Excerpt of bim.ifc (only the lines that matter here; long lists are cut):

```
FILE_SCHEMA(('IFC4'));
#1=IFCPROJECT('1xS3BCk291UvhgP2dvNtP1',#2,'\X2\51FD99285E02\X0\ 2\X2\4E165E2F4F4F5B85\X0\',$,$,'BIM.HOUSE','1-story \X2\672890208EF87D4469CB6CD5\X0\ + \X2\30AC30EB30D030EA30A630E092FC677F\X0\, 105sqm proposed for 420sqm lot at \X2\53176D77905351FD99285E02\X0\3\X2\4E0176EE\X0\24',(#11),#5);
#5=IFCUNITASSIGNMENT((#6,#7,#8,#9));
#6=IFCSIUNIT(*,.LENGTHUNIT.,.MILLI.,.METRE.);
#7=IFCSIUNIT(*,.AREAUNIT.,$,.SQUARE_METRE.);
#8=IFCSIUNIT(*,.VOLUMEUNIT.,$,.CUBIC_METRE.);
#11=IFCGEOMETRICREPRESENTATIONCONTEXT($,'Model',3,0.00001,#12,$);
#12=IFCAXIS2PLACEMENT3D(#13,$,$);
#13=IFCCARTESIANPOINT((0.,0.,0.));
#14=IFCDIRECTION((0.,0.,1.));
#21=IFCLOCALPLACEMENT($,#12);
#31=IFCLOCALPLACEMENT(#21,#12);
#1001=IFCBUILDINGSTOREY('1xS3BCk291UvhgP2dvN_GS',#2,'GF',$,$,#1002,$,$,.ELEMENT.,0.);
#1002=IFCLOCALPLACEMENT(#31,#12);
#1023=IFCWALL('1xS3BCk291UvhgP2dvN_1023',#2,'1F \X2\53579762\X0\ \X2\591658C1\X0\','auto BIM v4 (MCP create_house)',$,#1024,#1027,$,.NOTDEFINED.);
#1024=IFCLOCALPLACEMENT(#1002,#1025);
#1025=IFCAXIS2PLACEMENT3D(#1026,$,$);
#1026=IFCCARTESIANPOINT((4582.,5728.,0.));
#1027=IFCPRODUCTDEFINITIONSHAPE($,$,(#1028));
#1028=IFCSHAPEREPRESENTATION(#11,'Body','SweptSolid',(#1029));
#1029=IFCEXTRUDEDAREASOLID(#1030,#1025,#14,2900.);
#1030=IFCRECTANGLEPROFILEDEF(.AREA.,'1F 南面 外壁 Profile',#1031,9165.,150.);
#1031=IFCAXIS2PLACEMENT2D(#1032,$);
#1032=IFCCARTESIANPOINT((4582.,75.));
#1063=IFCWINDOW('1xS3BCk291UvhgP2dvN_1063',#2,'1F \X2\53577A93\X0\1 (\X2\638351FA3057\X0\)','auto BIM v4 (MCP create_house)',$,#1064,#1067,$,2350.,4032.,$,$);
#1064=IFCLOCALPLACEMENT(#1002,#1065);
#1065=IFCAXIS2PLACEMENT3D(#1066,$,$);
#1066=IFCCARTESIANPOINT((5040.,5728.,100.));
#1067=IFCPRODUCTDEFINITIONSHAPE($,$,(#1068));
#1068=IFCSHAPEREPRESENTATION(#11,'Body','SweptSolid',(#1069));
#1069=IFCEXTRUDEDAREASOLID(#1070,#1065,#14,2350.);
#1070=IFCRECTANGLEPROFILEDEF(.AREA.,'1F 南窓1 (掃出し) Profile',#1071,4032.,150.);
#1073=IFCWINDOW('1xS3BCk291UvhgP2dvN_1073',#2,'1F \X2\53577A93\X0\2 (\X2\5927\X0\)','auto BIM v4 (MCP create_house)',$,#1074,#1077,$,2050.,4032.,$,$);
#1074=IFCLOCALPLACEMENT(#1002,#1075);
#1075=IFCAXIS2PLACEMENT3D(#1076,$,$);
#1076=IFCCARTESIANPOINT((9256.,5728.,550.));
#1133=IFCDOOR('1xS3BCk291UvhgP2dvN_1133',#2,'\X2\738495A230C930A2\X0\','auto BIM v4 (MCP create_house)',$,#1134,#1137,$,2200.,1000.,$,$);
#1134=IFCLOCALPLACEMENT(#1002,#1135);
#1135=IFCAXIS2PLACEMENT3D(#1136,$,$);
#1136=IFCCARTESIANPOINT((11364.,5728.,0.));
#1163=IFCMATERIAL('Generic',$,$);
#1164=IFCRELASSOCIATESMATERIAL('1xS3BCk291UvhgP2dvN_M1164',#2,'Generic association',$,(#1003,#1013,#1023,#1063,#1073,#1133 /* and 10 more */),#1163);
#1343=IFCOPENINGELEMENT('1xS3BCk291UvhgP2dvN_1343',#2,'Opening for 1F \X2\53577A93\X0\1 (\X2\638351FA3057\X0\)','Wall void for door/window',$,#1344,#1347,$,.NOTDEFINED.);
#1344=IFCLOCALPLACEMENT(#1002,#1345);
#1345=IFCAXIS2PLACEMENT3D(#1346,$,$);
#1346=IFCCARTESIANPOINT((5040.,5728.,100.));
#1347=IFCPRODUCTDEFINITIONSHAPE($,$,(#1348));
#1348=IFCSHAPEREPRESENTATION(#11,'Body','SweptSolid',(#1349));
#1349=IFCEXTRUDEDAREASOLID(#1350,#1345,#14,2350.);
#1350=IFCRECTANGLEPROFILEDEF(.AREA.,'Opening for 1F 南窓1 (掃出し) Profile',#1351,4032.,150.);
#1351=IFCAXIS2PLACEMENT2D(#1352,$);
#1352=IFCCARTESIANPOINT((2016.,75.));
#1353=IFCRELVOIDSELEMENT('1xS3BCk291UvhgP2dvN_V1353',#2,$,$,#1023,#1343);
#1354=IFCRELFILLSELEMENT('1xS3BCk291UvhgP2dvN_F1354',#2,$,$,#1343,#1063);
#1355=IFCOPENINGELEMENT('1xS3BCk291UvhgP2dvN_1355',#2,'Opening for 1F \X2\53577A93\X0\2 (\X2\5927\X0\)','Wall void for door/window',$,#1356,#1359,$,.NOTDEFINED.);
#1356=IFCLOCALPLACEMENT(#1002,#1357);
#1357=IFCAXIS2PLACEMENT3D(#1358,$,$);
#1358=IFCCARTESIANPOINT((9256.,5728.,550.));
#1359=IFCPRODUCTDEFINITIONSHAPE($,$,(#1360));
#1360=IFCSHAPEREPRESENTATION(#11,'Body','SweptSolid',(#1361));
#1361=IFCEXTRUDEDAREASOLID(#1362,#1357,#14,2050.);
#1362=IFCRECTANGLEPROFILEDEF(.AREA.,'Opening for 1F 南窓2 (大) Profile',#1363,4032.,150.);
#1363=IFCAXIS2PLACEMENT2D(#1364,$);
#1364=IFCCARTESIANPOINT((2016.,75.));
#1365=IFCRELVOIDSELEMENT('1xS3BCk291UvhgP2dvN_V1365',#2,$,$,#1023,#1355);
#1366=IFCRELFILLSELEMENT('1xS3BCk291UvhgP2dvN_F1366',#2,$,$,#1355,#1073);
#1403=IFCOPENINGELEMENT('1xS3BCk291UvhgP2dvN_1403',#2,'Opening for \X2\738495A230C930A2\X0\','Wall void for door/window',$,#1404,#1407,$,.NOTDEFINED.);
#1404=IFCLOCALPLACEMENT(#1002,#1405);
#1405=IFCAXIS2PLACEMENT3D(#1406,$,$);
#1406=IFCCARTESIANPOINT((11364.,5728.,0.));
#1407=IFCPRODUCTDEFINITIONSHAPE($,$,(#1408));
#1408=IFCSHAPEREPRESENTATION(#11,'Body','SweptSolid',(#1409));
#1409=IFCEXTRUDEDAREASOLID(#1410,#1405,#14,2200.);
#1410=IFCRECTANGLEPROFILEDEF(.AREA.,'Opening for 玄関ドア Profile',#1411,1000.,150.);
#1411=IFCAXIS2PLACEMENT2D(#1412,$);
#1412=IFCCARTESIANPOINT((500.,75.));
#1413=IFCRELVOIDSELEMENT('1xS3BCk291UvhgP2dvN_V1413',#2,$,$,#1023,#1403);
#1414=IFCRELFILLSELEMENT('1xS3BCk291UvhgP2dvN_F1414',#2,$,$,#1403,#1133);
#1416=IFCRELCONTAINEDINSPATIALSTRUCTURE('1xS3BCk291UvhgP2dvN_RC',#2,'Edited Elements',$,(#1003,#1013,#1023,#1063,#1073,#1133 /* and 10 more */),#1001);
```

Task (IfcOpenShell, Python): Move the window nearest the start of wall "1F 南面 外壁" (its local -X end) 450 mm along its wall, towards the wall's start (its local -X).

```python
import ifcopenshell
import ifcopenshell.api.geometry
import ifcopenshell.util.placement

model = ifcopenshell.open("bim.ifc")

window = model.by_guid("1xS3BCk291UvhgP2dvN_1063")
opening = window.FillsVoids[0].RelatingOpeningElement
wall = opening.VoidsElements[0].RelatingBuildingElement

wall_matrix = ifcopenshell.util.placement.get_local_placement(wall.ObjectPlacement)
shift = wall_matrix[:3, 0] * -450.0
before = ifcopenshell.util.placement.get_local_placement(window.ObjectPlacement)[:3, 3].copy()

# The window is not placed relative to its opening, so move both.
for product in (opening, window):
    matrix = ifcopenshell.util.placement.get_local_placement(product.ObjectPlacement)
    matrix[:3, 3] += shift
    ifcopenshell.api.geometry.edit_object_placement(model, product=product, matrix=matrix, is_si=False)

after = ifcopenshell.util.placement.get_local_placement(window.ObjectPlacement)[:3, 3]
print("window moved by", (after - before).round(3) + 0.0)

model.write("bim_rev.ifc")
```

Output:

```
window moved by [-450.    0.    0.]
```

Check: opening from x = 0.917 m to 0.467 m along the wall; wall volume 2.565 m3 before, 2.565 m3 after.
